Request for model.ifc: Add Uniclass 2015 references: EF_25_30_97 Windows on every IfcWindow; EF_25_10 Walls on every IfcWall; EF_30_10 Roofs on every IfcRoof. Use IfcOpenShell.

First a look at what the model holds.

```python
import ifcopenshell

model = ifcopenshell.open("model.ifc")
print(model.schema)
print("classifications:", [c.Name for c in model.by_type("IfcClassification")])
for ifc_class in ("IfcDoor", "IfcRoof", "IfcStair", "IfcWall", "IfcWindow"):
    print(ifc_class, len(model.by_type(ifc_class)))
```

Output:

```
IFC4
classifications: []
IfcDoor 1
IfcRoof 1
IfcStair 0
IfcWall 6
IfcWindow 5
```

```python
import ifcopenshell
import ifcopenshell.api.classification

model = ifcopenshell.open("model.ifc")

system = ifcopenshell.api.classification.add_classification(model, classification="Uniclass 2015")

codes = {
    "IfcWindow": ("EF_25_30_97", "Windows"),
    "IfcWall": ("EF_25_10", "Walls"),
    "IfcRoof": ("EF_30_10", "Roofs"),
}
for ifc_class, (code, name) in codes.items():
    products = model.by_type(ifc_class)
    ifcopenshell.api.classification.add_reference(
        model, products=products, classification=system, identification=code, name=name
    )
    print(code, len(products))

model.write("model_v2.ifc")
```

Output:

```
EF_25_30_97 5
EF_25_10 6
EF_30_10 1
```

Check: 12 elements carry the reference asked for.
